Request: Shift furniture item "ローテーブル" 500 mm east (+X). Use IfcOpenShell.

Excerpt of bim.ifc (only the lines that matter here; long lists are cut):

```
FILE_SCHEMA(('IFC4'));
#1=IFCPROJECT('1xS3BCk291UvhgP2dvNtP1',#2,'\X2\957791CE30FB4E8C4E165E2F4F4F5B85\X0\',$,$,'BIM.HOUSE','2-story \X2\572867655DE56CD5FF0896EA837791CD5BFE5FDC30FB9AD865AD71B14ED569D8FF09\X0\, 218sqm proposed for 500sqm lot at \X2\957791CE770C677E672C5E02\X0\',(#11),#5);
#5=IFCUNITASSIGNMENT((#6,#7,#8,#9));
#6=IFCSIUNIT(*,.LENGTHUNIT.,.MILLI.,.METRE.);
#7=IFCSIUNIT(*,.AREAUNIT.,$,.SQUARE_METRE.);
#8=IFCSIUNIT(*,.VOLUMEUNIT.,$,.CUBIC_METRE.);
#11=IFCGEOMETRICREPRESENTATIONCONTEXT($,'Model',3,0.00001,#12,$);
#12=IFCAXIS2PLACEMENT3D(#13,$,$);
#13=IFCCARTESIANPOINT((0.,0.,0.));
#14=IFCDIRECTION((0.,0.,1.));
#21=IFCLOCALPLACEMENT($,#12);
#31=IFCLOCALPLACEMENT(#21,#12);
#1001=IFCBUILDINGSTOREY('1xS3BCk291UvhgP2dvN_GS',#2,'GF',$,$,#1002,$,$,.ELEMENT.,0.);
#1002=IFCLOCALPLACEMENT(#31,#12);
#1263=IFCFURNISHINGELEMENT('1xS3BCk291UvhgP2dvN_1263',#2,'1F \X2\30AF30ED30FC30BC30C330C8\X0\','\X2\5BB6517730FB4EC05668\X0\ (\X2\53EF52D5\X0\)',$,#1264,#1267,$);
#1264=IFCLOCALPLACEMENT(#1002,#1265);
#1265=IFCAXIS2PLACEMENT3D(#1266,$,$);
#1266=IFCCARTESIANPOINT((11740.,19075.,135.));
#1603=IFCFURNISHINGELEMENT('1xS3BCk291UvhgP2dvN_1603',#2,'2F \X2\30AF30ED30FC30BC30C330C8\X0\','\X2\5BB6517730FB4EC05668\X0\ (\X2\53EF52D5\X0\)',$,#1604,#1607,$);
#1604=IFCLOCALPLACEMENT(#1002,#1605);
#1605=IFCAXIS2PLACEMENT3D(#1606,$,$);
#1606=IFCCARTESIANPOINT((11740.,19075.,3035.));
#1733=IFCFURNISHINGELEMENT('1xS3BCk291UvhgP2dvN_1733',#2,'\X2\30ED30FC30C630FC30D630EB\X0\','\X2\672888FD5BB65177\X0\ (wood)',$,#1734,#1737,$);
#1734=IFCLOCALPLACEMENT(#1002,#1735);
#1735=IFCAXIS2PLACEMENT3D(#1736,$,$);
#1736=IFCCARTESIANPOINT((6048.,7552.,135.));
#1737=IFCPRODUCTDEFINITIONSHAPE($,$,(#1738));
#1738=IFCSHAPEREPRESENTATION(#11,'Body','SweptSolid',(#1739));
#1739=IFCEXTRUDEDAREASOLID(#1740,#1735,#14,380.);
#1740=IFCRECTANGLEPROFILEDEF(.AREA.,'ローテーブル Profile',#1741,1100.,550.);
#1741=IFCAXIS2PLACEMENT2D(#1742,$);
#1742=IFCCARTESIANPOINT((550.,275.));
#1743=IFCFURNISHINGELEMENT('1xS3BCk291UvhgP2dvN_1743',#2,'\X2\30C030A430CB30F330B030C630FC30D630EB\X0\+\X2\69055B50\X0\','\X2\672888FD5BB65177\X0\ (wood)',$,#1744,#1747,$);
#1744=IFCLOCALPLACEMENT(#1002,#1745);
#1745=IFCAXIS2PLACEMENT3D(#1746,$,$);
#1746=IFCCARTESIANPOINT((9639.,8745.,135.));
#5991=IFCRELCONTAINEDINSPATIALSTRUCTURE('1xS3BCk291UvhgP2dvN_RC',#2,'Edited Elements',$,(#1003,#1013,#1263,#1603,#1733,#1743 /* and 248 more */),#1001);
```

```python
import ifcopenshell
import ifcopenshell.api.geometry
import ifcopenshell.util.placement
import ifcopenshell.util.unit

model = ifcopenshell.open("bim.ifc")
unit_scale = ifcopenshell.util.unit.calculate_unit_scale(model)

item = model.by_guid("1xS3BCk291UvhgP2dvN_1733")
matrix = ifcopenshell.util.placement.get_local_placement(item.ObjectPlacement)
matrix[0, 3] += 0.5 / unit_scale
ifcopenshell.api.geometry.edit_object_placement(model, product=item, matrix=matrix, is_si=False)

print(ifcopenshell.util.placement.get_local_placement(item.ObjectPlacement).round(3) + 0.0)

model.write("bim_updated.ifc")
```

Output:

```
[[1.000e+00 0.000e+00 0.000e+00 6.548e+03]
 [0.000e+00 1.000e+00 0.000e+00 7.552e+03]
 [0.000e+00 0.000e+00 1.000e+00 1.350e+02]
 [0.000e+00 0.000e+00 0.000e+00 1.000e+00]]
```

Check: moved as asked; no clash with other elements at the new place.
